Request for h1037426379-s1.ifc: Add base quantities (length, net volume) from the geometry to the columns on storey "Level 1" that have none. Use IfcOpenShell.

First a look at what the model holds.

```python
import ifcopenshell
import ifcopenshell.util.element
import ifcopenshell.util.unit

model = ifcopenshell.open("h1037426379-s1.ifc")
print(model.schema)
for unit_type in ("LENGTHUNIT", "AREAUNIT", "VOLUMEUNIT"):
    print(unit_type, ifcopenshell.util.unit.calculate_unit_scale(model, unit_type))
storey = next(s for s in model.by_type("IfcBuildingStorey") if s.Name == "Level 1")
columns = [e for e in ifcopenshell.util.element.get_decomposition(storey) if e.is_a("IfcColumn")]
for e in sorted(columns, key=lambda e: e.id()):
    print(e.id(), e.is_a(), e.Name, list(ifcopenshell.util.element.get_psets(e, qtos_only=True)), sep=" | ")
```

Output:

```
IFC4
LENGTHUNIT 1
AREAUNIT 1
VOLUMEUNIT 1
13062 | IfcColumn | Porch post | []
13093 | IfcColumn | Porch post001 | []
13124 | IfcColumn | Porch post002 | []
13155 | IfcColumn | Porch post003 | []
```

```python
import ifcopenshell
import ifcopenshell.api.pset
import ifcopenshell.geom
import ifcopenshell.util.element
import ifcopenshell.util.shape
import ifcopenshell.util.unit

model = ifcopenshell.open("h1037426379-s1.ifc")
unit_scale = ifcopenshell.util.unit.calculate_unit_scale(model)
volume_scale = ifcopenshell.util.unit.calculate_unit_scale(model, "VOLUMEUNIT")
settings = ifcopenshell.geom.settings()

storey = next(s for s in model.by_type("IfcBuildingStorey") if s.Name == "Level 1")
columns = [e for e in ifcopenshell.util.element.get_decomposition(storey) if e.is_a("IfcColumn")]

for e in sorted(columns, key=lambda e: e.id()):
    if ifcopenshell.util.element.get_psets(e, qtos_only=True, should_inherit=False):
        continue
    # Geometry comes back in metres, in the element's own axes.
    shape = ifcopenshell.geom.create_shape(settings, e)
    values = {
        "Length": ifcopenshell.util.shape.get_z(shape.geometry) / unit_scale,
        "NetVolume": ifcopenshell.util.shape.get_volume(shape.geometry) / volume_scale,
    }
    qto = ifcopenshell.api.pset.add_qto(model, product=e, name="Qto_ColumnBaseQuantities")
    ifcopenshell.api.pset.edit_qto(model, qto=qto, properties=values)
    print(e.id(), {k: round(v, 3) for k, v in values.items()})

model.write("h1037426379-s1_edited.ifc")
```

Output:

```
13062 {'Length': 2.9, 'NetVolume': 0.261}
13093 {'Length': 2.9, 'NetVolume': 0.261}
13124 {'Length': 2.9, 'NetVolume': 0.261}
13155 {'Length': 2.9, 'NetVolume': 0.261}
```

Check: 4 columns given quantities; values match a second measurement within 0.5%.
